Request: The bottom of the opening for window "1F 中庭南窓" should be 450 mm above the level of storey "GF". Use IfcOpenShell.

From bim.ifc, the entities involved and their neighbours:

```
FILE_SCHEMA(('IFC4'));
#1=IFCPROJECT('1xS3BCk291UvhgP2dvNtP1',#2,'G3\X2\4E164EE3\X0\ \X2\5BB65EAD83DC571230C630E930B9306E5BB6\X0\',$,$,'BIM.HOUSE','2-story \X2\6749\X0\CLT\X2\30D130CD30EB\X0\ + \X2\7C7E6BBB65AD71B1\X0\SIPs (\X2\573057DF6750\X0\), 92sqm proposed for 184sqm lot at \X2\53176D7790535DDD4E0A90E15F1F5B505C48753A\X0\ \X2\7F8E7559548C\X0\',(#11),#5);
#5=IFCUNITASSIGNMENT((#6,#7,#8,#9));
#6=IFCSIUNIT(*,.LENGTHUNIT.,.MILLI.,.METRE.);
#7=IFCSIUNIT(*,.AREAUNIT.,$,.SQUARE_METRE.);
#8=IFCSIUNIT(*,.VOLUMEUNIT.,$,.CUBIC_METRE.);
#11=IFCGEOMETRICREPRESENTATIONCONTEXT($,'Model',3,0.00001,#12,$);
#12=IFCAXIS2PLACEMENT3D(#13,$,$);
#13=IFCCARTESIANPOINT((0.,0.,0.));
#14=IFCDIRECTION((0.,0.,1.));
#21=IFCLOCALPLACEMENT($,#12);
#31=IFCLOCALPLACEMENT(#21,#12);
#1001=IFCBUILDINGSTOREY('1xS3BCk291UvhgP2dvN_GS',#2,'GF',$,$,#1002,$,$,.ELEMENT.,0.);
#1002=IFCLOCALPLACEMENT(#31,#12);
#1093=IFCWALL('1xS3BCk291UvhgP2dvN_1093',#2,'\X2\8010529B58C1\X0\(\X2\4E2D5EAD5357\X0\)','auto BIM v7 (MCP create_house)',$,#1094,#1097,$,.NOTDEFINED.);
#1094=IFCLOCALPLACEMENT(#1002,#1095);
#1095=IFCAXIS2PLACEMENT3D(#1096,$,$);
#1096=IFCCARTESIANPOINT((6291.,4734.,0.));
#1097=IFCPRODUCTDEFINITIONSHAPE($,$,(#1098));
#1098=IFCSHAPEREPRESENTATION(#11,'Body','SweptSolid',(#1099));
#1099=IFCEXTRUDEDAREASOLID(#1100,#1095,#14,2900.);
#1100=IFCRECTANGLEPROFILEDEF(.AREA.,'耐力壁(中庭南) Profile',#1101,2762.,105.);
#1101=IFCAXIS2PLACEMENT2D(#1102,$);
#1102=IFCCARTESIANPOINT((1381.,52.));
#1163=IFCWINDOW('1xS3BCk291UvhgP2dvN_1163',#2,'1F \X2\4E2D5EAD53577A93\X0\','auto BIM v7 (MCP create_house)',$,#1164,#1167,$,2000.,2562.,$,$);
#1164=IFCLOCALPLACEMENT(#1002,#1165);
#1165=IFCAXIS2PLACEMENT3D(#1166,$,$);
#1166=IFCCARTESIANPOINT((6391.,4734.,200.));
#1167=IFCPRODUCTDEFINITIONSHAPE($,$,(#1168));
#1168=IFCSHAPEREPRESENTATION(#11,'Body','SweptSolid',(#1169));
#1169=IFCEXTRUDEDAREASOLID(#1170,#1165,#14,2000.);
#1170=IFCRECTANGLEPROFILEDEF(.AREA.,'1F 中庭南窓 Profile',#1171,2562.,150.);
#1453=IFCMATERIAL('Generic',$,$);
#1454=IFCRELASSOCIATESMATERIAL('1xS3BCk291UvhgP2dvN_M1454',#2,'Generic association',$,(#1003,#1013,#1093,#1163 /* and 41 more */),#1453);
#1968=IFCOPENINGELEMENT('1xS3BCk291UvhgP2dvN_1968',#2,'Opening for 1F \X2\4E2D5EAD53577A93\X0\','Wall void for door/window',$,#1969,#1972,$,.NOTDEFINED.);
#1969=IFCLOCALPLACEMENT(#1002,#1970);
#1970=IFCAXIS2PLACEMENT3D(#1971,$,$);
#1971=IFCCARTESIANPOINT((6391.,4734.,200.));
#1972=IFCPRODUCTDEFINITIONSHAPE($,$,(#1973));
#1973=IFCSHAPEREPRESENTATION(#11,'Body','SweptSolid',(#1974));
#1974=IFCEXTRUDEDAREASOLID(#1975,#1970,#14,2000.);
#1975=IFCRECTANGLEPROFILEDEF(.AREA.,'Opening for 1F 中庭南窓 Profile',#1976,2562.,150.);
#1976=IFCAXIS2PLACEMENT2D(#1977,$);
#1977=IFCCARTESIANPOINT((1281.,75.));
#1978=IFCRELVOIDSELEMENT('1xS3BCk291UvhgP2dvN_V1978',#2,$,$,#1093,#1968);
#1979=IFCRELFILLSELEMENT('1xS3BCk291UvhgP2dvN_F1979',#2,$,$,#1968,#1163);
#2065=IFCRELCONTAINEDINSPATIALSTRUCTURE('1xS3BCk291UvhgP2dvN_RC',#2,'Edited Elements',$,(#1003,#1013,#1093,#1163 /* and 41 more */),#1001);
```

```python
import numpy as np
import ifcopenshell
import ifcopenshell.api.geometry
import ifcopenshell.geom
import ifcopenshell.util.element
import ifcopenshell.util.placement
import ifcopenshell.util.shape
import ifcopenshell.util.unit

model = ifcopenshell.open("bim.ifc")
unit_scale = ifcopenshell.util.unit.calculate_unit_scale(model)

window = model.by_guid("1xS3BCk291UvhgP2dvN_1163")
opening = window.FillsVoids[0].RelatingOpeningElement
storey = ifcopenshell.util.element.get_container(window, ifc_class="IfcBuildingStorey")
level = ifcopenshell.util.placement.get_local_placement(storey.ObjectPlacement)[2, 3]

# The opening's origin need not be at the sill, so measure its lowest point.
shape = ifcopenshell.geom.create_shape(ifcopenshell.geom.settings(), opening)
bottom = ifcopenshell.util.shape.get_shape_bottom_elevation(shape, shape.geometry) / unit_scale
dz = level + 450.0 - bottom

shift = np.array([0.0, 0.0, dz])
# The window is not placed relative to its opening, so move both.
for product in (opening, window):
    matrix = ifcopenshell.util.placement.get_local_placement(product.ObjectPlacement)
    matrix[:3, 3] += shift
    ifcopenshell.api.geometry.edit_object_placement(model, product=product, matrix=matrix, is_si=False)

print(f"moved by {dz * unit_scale:+.3f} m")

model.write("bim_edited.ifc")
```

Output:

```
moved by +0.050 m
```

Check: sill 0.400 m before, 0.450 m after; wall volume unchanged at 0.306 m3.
